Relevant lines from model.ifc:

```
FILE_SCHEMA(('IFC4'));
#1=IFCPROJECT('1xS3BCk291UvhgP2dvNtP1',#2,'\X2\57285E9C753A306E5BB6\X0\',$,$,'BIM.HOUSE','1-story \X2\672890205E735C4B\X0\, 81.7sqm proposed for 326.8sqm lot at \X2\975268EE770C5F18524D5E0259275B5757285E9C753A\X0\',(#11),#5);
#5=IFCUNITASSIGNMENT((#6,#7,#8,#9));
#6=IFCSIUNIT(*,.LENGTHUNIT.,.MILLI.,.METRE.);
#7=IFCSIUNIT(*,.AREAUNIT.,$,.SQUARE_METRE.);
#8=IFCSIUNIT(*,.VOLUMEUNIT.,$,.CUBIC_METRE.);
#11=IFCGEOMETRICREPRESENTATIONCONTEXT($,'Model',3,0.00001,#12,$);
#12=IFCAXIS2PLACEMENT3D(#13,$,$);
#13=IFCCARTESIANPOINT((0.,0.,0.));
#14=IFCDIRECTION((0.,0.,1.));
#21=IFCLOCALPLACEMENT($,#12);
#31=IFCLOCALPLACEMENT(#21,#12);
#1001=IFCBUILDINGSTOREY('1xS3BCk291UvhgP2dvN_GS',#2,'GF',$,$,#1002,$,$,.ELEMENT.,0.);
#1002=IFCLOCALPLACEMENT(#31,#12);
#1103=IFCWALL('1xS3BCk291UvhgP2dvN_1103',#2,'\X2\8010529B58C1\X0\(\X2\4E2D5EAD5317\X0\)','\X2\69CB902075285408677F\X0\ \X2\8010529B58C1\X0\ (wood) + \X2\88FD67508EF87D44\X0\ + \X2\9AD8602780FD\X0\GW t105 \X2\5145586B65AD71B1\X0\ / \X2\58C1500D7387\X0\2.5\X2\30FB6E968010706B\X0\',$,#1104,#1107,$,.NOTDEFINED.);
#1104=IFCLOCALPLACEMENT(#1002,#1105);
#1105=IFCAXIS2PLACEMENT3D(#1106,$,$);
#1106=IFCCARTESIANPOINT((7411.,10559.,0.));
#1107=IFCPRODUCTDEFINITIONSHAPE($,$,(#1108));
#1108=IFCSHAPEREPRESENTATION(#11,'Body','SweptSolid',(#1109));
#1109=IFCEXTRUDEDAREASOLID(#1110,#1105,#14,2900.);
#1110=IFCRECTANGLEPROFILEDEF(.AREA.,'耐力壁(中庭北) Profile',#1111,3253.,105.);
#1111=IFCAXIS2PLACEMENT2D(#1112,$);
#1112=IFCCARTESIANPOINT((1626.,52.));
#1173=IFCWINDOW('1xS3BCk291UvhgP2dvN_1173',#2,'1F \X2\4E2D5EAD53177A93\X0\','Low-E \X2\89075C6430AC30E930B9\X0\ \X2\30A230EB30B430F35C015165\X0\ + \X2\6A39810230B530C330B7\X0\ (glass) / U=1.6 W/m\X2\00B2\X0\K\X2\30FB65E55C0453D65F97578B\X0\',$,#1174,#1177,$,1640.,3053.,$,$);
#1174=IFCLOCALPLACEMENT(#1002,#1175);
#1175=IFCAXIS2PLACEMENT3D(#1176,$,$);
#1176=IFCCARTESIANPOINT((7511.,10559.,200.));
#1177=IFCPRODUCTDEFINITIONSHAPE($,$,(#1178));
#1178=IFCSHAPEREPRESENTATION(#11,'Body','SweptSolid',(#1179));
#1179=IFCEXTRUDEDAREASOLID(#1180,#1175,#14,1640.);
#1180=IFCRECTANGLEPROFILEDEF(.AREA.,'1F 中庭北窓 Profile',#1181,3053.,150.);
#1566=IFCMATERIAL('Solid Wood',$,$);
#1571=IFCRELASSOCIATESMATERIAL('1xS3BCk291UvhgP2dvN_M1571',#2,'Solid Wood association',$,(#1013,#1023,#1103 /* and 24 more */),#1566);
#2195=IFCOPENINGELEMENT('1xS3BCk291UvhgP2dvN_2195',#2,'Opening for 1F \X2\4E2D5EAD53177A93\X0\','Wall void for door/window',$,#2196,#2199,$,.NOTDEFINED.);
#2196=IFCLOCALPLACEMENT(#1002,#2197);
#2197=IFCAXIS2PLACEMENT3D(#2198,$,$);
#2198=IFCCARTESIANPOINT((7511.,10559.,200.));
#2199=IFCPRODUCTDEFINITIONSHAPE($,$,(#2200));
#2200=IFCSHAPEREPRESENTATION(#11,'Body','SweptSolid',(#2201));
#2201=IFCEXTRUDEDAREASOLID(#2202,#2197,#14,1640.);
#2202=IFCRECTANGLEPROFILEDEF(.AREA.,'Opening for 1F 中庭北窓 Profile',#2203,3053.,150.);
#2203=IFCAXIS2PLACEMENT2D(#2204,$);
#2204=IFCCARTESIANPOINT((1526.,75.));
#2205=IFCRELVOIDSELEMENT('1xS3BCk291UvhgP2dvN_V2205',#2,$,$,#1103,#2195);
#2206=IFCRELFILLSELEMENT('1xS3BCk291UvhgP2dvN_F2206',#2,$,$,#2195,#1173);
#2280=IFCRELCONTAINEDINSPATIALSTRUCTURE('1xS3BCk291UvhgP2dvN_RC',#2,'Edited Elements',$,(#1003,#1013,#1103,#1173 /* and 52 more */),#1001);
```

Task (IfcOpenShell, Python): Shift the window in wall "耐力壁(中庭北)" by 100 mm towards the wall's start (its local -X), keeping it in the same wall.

```python
import ifcopenshell
import ifcopenshell.api.geometry
import ifcopenshell.util.placement
import ifcopenshell.util.unit

model = ifcopenshell.open("model.ifc")
unit_scale = ifcopenshell.util.unit.calculate_unit_scale(model)

window = model.by_guid("1xS3BCk291UvhgP2dvN_1173")
opening = window.FillsVoids[0].RelatingOpeningElement
wall = opening.VoidsElements[0].RelatingBuildingElement

wall_matrix = ifcopenshell.util.placement.get_local_placement(wall.ObjectPlacement)
shift = wall_matrix[:3, 0] * -0.1 / unit_scale
before = ifcopenshell.util.placement.get_local_placement(window.ObjectPlacement)[:3, 3].copy()

# The window is not placed relative to its opening, so move both.
for product in (opening, window):
    matrix = ifcopenshell.util.placement.get_local_placement(product.ObjectPlacement)
    matrix[:3, 3] += shift
    ifcopenshell.api.geometry.edit_object_placement(model, product=product, matrix=matrix, is_si=False)

after = ifcopenshell.util.placement.get_local_placement(window.ObjectPlacement)[:3, 3]
print("window moved by", (after - before).round(3) + 0.0)

model.write("model_rev.ifc")
```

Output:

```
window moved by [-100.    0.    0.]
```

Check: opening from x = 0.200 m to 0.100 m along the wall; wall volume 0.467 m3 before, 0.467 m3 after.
